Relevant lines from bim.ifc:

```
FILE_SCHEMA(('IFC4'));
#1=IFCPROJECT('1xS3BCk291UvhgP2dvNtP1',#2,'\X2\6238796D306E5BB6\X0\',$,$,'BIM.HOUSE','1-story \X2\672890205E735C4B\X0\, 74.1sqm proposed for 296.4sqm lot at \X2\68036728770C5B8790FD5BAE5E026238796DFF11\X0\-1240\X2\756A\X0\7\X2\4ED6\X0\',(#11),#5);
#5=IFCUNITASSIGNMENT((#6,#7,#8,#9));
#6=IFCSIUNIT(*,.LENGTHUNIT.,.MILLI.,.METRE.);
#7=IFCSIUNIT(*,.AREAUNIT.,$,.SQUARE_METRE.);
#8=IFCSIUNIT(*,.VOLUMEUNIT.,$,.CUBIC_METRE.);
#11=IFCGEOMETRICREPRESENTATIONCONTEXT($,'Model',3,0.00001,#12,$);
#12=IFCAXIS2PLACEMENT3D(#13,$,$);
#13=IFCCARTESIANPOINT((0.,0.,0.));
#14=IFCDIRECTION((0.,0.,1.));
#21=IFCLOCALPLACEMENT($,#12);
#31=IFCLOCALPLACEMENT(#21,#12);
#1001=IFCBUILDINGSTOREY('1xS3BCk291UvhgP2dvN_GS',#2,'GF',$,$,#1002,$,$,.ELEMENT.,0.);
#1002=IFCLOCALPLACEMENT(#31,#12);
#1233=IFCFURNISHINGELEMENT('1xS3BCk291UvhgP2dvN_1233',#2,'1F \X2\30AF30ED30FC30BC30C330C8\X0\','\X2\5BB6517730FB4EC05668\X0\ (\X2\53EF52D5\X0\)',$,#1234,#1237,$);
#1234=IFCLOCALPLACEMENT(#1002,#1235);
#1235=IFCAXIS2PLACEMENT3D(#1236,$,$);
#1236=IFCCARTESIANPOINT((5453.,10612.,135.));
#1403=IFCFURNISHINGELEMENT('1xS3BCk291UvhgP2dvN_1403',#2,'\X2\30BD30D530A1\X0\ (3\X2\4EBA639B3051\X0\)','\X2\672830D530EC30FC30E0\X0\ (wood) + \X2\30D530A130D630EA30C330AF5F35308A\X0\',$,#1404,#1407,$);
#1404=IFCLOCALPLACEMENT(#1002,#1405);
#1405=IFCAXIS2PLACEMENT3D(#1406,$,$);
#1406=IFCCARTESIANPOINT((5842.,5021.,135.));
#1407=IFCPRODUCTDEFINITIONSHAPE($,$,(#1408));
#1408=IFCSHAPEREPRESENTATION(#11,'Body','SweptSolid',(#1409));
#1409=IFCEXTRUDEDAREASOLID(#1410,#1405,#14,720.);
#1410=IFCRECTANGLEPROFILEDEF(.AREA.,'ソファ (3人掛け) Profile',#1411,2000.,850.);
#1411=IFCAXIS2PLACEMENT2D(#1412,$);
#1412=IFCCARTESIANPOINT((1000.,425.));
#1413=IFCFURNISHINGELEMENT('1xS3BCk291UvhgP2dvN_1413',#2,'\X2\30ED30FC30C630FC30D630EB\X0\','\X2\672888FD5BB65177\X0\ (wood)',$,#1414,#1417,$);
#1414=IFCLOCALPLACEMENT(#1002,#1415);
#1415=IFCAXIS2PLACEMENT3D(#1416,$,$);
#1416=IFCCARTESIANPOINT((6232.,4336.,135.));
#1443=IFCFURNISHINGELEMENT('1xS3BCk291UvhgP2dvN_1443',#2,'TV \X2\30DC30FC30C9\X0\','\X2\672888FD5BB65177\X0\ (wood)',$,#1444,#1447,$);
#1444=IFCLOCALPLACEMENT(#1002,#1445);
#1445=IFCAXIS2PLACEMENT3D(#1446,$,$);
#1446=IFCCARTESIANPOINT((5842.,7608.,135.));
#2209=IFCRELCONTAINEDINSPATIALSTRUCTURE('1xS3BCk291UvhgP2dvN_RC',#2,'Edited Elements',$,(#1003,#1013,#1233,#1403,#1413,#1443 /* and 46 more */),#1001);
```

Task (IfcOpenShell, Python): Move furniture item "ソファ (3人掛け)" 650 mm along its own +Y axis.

```python
import ifcopenshell
import ifcopenshell.api.geometry
import ifcopenshell.util.placement
import ifcopenshell.util.unit

model = ifcopenshell.open("bim.ifc")
unit_scale = ifcopenshell.util.unit.calculate_unit_scale(model)

item = model.by_guid("1xS3BCk291UvhgP2dvN_1403")
matrix = ifcopenshell.util.placement.get_local_placement(item.ObjectPlacement)
matrix[:3, 3] += matrix[:3, 1] * 0.65 / unit_scale
ifcopenshell.api.geometry.edit_object_placement(model, product=item, matrix=matrix, is_si=False)

print(ifcopenshell.util.placement.get_local_placement(item.ObjectPlacement).round(3) + 0.0)

model.write("bim_updated.ifc")
```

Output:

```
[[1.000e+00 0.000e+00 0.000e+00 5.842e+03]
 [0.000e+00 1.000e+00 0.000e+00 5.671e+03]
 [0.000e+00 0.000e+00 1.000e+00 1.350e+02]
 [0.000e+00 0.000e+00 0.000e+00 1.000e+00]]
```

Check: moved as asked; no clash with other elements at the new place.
